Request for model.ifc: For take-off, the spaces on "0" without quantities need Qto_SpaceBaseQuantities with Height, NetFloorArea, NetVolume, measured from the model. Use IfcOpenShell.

First a look at what the model holds.

```python
import ifcopenshell
import ifcopenshell.util.element
import ifcopenshell.util.unit

model = ifcopenshell.open("model.ifc")
print(model.schema)
for unit_type in ("LENGTHUNIT", "AREAUNIT", "VOLUMEUNIT"):
    print(unit_type, ifcopenshell.util.unit.calculate_unit_scale(model, unit_type))
storey = next(s for s in model.by_type("IfcBuildingStorey") if s.Name == "0")
spaces = [e for e in ifcopenshell.util.element.get_decomposition(storey) if e.is_a("IfcSpace")]
for e in sorted(spaces, key=lambda e: e.id()):
    print(e.id(), e.is_a(), e.Name, list(ifcopenshell.util.element.get_psets(e, qtos_only=True)), sep=" | ")
```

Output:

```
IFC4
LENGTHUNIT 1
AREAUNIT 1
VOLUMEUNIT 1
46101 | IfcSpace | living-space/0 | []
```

```python
import ifcopenshell
import ifcopenshell.api.pset
import ifcopenshell.geom
import ifcopenshell.util.element
import ifcopenshell.util.shape
import ifcopenshell.util.unit

model = ifcopenshell.open("model.ifc")
unit_scale = ifcopenshell.util.unit.calculate_unit_scale(model)
area_scale = ifcopenshell.util.unit.calculate_unit_scale(model, "AREAUNIT")
volume_scale = ifcopenshell.util.unit.calculate_unit_scale(model, "VOLUMEUNIT")
settings = ifcopenshell.geom.settings()

storey = next(s for s in model.by_type("IfcBuildingStorey") if s.Name == "0")
spaces = [e for e in ifcopenshell.util.element.get_decomposition(storey) if e.is_a("IfcSpace")]

for e in sorted(spaces, key=lambda e: e.id()):
    if ifcopenshell.util.element.get_psets(e, qtos_only=True, should_inherit=False):
        continue
    # Geometry comes back in metres, in the element's own axes.
    shape = ifcopenshell.geom.create_shape(settings, e)
    values = {
        "Height": ifcopenshell.util.shape.get_z(shape.geometry) / unit_scale,
        "NetFloorArea": ifcopenshell.util.shape.get_footprint_area(shape.geometry) / area_scale,
        "NetVolume": ifcopenshell.util.shape.get_volume(shape.geometry) / volume_scale,
    }
    qto = ifcopenshell.api.pset.add_qto(model, product=e, name="Qto_SpaceBaseQuantities")
    ifcopenshell.api.pset.edit_qto(model, qto=qto, properties=values)
    print(e.id(), {k: round(v, 3) for k, v in values.items()})

model.write("model_edited.ifc")
```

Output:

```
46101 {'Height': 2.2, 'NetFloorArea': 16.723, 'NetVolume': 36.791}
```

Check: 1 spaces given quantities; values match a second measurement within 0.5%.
